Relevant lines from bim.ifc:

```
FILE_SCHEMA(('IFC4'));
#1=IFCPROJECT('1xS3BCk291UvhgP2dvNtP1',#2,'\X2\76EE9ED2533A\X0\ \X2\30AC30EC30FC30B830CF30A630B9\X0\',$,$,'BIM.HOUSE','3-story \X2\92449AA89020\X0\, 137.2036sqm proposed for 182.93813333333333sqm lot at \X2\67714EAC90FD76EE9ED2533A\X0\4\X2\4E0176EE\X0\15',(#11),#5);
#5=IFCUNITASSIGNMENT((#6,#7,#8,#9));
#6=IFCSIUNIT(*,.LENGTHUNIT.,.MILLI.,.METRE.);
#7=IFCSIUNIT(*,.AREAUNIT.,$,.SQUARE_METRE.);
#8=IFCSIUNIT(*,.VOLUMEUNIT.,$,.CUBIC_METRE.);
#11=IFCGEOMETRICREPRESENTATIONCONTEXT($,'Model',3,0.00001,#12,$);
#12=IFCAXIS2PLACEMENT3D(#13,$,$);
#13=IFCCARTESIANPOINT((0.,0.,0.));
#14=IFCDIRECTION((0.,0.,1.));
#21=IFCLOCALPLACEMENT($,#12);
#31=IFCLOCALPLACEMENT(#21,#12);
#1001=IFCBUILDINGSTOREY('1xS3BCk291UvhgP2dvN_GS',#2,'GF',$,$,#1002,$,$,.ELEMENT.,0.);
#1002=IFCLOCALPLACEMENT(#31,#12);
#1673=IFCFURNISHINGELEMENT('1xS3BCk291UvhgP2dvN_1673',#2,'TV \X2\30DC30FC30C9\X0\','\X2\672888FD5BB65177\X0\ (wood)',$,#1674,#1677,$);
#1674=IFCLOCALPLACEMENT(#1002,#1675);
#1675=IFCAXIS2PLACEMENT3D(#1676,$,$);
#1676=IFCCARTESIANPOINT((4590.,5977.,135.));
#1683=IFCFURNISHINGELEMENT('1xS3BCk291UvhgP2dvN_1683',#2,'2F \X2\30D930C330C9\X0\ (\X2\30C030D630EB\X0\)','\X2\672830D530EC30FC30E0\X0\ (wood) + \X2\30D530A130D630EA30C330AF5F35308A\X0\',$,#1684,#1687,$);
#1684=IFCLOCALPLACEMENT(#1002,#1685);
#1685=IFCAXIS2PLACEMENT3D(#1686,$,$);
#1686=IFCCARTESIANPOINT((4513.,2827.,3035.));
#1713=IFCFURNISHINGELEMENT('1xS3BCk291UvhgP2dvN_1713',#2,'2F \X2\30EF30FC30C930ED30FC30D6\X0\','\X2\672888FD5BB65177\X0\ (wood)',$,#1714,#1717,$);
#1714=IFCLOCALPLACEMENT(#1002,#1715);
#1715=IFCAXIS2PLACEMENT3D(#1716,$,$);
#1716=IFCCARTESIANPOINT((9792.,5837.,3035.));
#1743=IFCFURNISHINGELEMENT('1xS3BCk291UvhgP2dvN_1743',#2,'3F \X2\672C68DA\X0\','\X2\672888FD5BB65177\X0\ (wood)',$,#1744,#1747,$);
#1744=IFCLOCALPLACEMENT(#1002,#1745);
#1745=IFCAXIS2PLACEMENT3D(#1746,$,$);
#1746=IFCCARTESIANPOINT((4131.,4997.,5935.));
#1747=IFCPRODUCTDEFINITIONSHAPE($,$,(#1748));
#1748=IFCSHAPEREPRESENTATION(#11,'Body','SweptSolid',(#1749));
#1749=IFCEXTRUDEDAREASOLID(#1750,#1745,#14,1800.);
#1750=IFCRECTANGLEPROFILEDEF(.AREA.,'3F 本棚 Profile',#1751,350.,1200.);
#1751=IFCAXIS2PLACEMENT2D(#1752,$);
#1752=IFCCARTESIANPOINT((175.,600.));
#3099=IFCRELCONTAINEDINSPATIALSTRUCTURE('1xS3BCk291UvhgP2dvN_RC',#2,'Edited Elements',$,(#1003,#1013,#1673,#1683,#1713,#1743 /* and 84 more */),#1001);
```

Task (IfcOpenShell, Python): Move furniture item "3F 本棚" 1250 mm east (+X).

```python
import ifcopenshell
import ifcopenshell.api.geometry
import ifcopenshell.util.placement

model = ifcopenshell.open("bim.ifc")

item = model.by_id(1743)
matrix = ifcopenshell.util.placement.get_local_placement(item.ObjectPlacement)
matrix[0, 3] += 1250.0
ifcopenshell.api.geometry.edit_object_placement(model, product=item, matrix=matrix, is_si=False)

print(ifcopenshell.util.placement.get_local_placement(item.ObjectPlacement).round(3) + 0.0)

model.write("bim-out.ifc")
```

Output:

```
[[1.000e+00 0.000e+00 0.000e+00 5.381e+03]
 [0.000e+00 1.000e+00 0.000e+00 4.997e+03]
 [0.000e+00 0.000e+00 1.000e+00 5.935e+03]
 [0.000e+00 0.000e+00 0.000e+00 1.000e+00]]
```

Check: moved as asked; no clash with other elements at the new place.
